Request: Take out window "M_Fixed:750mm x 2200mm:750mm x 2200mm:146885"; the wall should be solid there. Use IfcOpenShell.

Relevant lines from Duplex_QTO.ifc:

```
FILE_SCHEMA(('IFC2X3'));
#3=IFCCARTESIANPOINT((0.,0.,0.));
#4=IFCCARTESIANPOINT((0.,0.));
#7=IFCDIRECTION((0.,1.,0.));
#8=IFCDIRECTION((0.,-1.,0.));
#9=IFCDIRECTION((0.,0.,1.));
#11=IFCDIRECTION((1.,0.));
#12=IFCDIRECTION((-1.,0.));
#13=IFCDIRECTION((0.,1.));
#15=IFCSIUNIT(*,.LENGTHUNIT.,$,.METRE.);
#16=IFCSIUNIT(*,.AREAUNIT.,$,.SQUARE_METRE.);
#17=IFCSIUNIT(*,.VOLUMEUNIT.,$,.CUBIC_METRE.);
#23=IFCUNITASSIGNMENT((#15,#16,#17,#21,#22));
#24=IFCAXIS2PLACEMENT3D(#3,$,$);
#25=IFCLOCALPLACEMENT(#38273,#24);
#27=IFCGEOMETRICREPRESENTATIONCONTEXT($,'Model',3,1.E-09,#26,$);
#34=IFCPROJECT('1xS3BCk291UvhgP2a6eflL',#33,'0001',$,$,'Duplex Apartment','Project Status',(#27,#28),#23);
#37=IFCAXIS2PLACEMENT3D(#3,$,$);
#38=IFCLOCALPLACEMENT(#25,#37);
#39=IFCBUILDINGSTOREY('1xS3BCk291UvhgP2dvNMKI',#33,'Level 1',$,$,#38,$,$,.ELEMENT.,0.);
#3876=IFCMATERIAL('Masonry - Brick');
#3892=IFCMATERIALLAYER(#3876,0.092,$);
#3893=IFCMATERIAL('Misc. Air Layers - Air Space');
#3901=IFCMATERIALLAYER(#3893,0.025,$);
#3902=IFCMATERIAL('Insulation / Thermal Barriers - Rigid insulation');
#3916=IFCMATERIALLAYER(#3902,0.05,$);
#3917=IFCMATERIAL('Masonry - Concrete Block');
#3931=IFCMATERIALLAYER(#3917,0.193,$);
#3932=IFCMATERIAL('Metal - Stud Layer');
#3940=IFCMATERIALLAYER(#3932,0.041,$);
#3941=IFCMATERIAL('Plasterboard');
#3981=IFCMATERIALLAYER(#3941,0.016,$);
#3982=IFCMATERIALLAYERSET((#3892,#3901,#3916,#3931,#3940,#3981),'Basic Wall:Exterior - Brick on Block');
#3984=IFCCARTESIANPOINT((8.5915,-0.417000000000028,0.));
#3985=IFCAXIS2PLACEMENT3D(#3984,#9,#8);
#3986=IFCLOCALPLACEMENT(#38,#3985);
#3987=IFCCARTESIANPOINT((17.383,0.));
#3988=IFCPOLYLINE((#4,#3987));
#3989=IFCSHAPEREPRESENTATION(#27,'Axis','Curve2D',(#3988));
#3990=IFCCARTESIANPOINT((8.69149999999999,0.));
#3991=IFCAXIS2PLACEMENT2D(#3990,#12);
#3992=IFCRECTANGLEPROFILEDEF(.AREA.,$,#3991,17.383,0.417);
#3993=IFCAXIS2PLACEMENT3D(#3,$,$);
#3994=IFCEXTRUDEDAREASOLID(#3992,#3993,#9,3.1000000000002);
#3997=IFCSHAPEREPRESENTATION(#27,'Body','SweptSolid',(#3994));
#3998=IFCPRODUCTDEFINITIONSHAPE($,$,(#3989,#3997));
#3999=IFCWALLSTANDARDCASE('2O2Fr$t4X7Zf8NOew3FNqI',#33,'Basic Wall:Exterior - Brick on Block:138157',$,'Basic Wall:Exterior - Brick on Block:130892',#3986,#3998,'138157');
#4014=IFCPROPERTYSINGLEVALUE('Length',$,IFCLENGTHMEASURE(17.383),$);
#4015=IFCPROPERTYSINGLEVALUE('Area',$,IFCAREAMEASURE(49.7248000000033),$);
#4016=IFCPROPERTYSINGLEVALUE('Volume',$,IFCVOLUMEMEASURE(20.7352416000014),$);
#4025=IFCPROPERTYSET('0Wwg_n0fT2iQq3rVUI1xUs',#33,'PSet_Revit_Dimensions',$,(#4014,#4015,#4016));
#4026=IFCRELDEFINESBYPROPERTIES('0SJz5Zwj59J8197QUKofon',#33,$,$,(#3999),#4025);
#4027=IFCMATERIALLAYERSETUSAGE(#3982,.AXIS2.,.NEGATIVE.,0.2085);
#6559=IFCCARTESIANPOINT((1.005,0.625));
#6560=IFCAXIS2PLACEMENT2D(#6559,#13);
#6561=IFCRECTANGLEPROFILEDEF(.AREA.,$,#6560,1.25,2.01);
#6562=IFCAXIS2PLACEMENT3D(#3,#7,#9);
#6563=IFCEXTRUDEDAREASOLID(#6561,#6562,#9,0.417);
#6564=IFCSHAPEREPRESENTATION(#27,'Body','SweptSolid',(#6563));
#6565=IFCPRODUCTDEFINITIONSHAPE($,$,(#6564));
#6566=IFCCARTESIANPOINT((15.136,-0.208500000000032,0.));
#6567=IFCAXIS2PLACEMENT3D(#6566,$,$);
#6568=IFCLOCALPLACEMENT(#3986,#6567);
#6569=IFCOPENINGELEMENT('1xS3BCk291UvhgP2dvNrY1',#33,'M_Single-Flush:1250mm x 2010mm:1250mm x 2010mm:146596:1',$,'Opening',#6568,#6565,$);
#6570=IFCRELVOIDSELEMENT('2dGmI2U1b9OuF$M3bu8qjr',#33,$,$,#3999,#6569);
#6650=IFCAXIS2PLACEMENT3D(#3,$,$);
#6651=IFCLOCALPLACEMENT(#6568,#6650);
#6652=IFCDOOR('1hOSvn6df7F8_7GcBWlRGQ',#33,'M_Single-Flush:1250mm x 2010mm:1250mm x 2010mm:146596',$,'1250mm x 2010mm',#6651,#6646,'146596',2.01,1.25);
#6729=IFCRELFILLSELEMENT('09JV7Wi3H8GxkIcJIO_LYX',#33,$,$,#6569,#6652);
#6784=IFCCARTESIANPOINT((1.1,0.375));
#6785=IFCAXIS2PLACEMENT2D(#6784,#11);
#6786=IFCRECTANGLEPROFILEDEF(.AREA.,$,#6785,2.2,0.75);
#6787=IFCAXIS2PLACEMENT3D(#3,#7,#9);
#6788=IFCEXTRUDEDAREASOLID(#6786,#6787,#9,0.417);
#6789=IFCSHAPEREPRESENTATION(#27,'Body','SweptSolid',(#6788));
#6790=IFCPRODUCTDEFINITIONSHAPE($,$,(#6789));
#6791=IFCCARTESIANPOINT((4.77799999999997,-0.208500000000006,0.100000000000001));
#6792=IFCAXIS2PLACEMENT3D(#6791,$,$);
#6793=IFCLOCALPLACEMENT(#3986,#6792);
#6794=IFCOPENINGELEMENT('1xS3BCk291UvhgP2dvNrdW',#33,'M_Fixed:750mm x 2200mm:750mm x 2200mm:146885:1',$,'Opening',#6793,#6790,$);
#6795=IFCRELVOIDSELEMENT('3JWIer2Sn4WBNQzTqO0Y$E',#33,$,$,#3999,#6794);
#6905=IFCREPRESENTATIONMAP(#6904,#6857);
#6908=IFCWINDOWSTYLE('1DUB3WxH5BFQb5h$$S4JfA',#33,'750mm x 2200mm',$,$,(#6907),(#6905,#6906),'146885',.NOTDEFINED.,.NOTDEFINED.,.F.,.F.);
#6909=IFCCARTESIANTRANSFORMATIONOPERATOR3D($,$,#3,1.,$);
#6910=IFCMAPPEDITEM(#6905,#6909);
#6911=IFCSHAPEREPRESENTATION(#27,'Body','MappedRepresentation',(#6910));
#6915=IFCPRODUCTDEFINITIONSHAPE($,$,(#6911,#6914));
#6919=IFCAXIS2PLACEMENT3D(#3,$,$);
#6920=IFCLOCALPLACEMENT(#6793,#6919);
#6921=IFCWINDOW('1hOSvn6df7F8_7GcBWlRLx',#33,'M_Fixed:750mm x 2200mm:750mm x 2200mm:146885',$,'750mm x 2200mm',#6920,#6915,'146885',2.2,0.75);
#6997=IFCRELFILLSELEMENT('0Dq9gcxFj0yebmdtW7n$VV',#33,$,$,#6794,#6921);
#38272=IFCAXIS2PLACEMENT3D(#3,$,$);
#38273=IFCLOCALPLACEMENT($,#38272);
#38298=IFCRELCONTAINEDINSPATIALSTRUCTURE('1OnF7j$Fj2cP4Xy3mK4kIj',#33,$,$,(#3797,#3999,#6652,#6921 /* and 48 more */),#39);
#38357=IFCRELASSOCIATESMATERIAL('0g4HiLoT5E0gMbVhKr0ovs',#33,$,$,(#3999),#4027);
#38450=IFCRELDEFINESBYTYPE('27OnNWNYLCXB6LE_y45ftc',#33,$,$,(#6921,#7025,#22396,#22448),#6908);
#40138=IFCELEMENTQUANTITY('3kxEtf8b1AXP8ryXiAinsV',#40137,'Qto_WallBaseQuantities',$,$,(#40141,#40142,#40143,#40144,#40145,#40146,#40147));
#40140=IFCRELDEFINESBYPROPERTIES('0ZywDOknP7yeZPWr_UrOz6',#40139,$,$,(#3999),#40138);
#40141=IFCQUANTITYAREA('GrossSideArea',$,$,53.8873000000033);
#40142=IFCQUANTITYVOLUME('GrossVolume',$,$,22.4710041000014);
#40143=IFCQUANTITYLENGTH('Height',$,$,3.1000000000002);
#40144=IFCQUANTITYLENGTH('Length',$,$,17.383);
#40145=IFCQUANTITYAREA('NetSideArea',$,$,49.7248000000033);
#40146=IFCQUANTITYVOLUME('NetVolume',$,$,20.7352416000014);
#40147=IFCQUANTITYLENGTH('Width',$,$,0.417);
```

```python
import ifcopenshell
import ifcopenshell.api.feature
import ifcopenshell.api.pset
import ifcopenshell.api.root
import ifcopenshell.geom
import ifcopenshell.util.element
import ifcopenshell.util.shape
import ifcopenshell.util.unit

model = ifcopenshell.open("Duplex_QTO.ifc")
area_scale = ifcopenshell.util.unit.calculate_unit_scale(model, "AREAUNIT")
volume_scale = ifcopenshell.util.unit.calculate_unit_scale(model, "VOLUMEUNIT")
settings = ifcopenshell.geom.settings()


def volume(element):
    """Net volume in cubic metres, openings subtracted."""
    shape = ifcopenshell.geom.create_shape(settings, element)
    return ifcopenshell.util.shape.get_volume(shape.geometry)


window = model.by_id(6921)
opening = window.FillsVoids[0].RelatingOpeningElement
wall = opening.VoidsElements[0].RelatingBuildingElement
before = volume(wall)

ifcopenshell.api.root.remove_product(model, product=window)
ifcopenshell.api.feature.remove_feature(model, feature=opening)

after = volume(wall)
thickness = 0.417  # wall thickness in metres

# Update the wall's stored quantities.
pset = model.by_id(ifcopenshell.util.element.get_pset(wall, "PSet_Revit_Dimensions", should_inherit=False)["id"])
ifcopenshell.api.pset.edit_pset(model, pset=pset, properties={
    "Area": model.create_entity("IfcAreaMeasure", after / thickness / area_scale),
    "Volume": model.create_entity("IfcVolumeMeasure", after / volume_scale),
})
qto = model.by_id(ifcopenshell.util.element.get_pset(wall, "Qto_WallBaseQuantities", should_inherit=False)["id"])
ifcopenshell.api.pset.edit_qto(model, qto=qto, properties={
    "NetSideArea": after / thickness / area_scale,
    "NetVolume": after / volume_scale,
})

print(f"wall volume {before:.3f} -> {after:.3f} m3")

model.write("Duplex_QTO_edited.ifc")
```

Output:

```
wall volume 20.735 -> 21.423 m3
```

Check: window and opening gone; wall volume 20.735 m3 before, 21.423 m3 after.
